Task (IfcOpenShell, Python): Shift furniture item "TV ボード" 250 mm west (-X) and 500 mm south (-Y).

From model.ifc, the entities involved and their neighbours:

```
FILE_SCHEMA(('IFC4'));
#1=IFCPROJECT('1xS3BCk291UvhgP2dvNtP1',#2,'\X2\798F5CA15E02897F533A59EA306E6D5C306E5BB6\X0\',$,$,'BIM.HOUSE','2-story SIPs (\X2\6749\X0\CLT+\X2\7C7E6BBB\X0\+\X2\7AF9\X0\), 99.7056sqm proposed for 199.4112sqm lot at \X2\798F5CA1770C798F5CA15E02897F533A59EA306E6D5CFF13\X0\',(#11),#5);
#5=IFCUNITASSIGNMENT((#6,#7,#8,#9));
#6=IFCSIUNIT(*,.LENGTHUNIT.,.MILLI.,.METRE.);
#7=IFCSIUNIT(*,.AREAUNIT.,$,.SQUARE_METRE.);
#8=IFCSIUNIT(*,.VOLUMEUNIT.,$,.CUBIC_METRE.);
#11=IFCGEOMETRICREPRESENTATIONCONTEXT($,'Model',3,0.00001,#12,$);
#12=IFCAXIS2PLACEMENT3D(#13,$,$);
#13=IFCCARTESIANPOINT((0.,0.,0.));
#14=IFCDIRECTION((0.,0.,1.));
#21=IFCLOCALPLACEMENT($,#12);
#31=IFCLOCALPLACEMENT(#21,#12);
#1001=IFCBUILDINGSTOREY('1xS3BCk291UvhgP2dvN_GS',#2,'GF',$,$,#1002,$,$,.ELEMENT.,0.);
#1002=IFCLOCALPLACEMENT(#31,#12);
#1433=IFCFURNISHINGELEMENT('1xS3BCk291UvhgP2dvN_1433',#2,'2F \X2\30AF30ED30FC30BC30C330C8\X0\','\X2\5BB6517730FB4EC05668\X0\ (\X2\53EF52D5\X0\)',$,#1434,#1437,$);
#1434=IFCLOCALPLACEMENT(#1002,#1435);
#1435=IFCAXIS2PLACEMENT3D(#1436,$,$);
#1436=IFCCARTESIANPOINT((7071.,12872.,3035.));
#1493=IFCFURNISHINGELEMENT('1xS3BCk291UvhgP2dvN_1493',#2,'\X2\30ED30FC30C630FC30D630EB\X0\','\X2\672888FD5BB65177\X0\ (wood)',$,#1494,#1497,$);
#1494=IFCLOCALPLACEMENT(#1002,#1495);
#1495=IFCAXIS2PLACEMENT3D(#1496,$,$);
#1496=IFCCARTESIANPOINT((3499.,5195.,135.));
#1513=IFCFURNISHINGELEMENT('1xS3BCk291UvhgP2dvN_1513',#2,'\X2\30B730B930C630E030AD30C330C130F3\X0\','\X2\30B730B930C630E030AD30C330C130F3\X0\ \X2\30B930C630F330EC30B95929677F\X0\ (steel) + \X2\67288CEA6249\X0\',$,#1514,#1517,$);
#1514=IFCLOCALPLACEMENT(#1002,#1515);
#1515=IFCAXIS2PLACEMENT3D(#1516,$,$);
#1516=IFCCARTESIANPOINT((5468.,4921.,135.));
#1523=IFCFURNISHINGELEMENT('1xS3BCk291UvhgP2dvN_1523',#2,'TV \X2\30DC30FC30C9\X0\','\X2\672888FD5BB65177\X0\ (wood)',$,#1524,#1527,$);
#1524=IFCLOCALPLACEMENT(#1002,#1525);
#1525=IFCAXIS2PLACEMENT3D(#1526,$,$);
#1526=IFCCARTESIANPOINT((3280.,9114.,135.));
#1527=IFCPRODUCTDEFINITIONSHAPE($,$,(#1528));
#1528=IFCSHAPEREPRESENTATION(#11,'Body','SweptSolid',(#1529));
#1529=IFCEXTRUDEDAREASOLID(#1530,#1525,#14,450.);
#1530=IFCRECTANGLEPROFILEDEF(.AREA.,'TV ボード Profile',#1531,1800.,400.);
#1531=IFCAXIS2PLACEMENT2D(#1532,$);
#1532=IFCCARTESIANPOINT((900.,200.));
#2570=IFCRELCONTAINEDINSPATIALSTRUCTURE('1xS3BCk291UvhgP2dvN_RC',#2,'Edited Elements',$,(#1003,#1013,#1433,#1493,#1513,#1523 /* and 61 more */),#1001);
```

```python
import ifcopenshell
import ifcopenshell.api.geometry
import ifcopenshell.util.placement

model = ifcopenshell.open("model.ifc")

item = model.by_guid("1xS3BCk291UvhgP2dvN_1523")
matrix = ifcopenshell.util.placement.get_local_placement(item.ObjectPlacement)
matrix[0, 3] -= 250.0
matrix[1, 3] -= 500.0
ifcopenshell.api.geometry.edit_object_placement(model, product=item, matrix=matrix, is_si=False)

print(ifcopenshell.util.placement.get_local_placement(item.ObjectPlacement).round(3) + 0.0)

model.write("model-out.ifc")
```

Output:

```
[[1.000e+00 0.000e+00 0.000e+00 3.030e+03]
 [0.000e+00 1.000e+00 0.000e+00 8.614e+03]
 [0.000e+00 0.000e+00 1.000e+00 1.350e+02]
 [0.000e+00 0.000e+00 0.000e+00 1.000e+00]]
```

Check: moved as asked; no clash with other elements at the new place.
